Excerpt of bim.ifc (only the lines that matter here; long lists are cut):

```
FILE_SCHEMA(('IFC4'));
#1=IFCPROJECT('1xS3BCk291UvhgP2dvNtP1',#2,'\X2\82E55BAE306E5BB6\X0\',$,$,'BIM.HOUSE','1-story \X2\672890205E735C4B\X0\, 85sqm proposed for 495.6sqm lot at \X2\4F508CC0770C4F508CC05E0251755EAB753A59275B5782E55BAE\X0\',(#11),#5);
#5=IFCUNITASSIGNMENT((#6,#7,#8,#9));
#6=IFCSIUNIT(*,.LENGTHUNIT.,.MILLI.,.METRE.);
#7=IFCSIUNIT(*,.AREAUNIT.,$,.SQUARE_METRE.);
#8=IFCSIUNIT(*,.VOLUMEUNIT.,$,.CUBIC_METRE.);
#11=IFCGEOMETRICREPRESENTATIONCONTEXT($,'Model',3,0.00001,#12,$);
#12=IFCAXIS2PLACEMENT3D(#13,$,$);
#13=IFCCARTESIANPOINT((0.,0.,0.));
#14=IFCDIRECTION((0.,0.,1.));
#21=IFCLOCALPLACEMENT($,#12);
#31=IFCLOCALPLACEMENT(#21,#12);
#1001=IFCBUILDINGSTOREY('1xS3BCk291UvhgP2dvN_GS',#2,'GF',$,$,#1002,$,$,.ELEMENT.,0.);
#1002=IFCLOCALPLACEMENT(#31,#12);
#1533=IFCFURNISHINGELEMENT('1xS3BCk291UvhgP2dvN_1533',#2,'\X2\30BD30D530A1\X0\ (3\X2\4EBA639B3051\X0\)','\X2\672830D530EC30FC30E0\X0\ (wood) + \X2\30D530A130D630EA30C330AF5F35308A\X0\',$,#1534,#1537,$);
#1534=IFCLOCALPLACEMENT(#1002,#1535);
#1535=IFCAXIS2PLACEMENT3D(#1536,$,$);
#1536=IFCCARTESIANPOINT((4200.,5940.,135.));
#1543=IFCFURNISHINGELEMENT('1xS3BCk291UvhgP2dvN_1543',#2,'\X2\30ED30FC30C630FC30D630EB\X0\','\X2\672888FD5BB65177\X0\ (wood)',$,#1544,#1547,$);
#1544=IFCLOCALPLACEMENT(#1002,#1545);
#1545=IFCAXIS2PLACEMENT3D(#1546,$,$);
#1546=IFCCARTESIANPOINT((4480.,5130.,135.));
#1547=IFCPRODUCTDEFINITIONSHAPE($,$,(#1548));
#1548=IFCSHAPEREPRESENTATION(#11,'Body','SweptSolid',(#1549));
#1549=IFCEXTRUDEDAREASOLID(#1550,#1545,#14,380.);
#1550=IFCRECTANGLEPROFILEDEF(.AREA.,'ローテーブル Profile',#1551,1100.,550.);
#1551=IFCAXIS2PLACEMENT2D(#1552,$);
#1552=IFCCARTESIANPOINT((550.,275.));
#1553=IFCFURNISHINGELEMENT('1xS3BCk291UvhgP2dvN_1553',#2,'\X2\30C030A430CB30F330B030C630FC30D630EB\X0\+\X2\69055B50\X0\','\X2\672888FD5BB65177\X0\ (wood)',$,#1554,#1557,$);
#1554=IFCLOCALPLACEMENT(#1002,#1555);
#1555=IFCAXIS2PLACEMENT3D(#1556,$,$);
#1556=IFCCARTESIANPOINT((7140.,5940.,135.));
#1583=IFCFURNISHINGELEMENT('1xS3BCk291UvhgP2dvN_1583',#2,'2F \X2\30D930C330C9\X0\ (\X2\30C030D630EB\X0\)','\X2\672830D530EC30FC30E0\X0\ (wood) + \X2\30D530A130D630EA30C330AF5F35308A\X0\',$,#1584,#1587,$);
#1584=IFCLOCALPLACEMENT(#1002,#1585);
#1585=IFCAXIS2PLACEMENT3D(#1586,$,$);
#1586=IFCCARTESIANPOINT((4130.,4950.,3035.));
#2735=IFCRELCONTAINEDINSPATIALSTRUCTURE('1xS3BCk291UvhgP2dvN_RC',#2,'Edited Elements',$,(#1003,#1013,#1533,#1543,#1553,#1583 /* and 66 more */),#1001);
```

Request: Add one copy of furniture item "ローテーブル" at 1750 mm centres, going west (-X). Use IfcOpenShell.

```python
import numpy as np
import ifcopenshell
import ifcopenshell.api.geometry
import ifcopenshell.api.root
import ifcopenshell.util.element
import ifcopenshell.util.placement
import ifcopenshell.util.unit

model = ifcopenshell.open("bim.ifc")
unit_scale = ifcopenshell.util.unit.calculate_unit_scale(model)


def reuse_history(source, copy):
    """copy_class also copies each property set's owner history, people and application; keep the originals."""
    for rel in copy.IsDefinedBy:
        if rel.is_a("IfcRelDefinesByProperties") and (history := rel.RelatingPropertyDefinition.OwnerHistory):
            rel.RelatingPropertyDefinition.OwnerHistory = source.OwnerHistory
            ifcopenshell.util.element.remove_deep2(model, history)


source = model.by_id(1543)
base = ifcopenshell.util.placement.get_local_placement(source.ObjectPlacement)
step = np.array([-1.0, 0.0, 0.0]) * 1.75 / unit_scale

for i in range(1, 2):
    copy = ifcopenshell.api.root.copy_class(model, product=source)
    copy.Representation = ifcopenshell.util.element.copy_deep(
        model, source.Representation, exclude=["IfcGeometricRepresentationContext", "IfcRepresentationMap"]
    )
    reuse_history(source, copy)
    matrix = base.copy()
    matrix[:3, 3] += i * step
    print("added at", matrix[:3, 3].round(3) + 0.0)
    ifcopenshell.api.geometry.edit_object_placement(model, product=copy, matrix=matrix, is_si=False)

model.write("bim_v2.ifc")
```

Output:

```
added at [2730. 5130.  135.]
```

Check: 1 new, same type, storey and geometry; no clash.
